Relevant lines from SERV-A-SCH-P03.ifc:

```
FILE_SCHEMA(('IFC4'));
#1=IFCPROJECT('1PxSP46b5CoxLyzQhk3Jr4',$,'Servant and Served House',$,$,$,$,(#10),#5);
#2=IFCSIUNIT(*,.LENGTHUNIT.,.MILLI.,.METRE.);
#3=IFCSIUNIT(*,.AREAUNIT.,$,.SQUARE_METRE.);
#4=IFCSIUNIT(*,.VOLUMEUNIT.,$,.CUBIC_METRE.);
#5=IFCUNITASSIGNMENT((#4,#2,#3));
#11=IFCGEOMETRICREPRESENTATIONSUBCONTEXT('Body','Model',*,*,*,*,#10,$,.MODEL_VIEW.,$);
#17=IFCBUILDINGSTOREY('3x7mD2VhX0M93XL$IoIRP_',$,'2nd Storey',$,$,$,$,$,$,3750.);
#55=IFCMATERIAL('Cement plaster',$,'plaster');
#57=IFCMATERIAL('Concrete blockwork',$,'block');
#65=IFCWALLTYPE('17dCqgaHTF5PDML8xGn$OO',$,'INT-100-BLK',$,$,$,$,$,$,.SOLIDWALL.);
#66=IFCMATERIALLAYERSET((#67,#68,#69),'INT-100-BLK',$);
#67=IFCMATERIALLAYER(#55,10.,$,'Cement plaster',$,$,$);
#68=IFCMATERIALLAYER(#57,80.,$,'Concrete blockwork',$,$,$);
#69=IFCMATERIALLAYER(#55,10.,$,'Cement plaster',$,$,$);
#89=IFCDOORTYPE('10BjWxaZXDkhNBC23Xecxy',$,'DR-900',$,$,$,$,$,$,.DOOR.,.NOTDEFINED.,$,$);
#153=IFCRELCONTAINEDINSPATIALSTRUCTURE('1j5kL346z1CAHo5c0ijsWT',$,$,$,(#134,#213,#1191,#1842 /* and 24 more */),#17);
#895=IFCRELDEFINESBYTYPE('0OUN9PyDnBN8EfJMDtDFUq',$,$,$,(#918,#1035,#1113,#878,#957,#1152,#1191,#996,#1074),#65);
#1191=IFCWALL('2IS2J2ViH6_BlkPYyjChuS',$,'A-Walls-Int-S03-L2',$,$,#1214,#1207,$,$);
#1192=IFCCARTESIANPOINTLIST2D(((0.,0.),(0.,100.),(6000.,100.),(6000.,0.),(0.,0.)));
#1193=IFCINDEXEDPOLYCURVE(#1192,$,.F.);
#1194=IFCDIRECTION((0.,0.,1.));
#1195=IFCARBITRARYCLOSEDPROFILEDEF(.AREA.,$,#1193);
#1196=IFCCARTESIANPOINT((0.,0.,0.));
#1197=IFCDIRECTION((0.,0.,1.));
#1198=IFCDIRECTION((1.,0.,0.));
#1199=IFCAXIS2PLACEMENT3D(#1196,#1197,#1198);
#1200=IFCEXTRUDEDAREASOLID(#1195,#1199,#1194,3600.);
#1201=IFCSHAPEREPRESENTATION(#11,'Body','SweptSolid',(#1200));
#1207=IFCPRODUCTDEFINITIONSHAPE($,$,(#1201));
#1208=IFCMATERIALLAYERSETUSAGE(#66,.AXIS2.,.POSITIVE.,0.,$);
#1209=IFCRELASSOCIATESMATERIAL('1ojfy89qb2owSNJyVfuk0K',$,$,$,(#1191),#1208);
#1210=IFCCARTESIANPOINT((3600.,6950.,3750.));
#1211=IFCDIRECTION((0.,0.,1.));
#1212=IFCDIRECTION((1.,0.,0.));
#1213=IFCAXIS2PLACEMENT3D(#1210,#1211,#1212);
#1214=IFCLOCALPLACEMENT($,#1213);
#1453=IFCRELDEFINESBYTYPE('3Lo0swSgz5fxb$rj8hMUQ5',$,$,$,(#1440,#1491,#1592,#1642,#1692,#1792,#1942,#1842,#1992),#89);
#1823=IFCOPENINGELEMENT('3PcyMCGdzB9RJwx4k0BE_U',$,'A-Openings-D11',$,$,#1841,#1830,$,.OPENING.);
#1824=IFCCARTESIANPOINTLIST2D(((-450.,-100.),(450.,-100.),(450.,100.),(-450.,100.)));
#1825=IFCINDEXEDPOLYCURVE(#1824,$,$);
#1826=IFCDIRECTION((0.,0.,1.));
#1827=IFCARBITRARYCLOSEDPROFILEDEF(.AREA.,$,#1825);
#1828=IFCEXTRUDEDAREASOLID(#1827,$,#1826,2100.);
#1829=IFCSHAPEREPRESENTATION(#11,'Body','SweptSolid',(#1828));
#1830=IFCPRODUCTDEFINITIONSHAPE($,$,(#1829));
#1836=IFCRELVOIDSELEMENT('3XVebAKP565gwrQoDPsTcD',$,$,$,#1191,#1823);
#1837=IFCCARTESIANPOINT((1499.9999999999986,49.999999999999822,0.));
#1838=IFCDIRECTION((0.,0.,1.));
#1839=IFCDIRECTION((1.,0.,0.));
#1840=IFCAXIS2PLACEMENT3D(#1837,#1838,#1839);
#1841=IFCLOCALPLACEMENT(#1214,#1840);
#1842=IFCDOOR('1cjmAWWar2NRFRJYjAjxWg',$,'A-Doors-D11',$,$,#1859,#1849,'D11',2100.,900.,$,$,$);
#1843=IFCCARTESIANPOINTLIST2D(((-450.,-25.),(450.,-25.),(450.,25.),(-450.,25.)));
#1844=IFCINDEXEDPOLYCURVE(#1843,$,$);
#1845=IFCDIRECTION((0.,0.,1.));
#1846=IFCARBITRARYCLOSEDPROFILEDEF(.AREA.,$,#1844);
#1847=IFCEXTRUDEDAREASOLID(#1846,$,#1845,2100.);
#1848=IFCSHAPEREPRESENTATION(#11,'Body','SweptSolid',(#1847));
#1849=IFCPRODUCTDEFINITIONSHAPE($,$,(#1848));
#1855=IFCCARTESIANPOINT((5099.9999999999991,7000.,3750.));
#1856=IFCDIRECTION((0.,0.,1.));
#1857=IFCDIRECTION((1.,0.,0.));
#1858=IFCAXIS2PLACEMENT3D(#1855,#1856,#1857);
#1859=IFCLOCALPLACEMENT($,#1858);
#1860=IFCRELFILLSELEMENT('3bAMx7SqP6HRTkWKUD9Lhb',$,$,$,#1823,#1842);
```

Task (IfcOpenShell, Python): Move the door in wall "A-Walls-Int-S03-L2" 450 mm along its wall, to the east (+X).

```python
import ifcopenshell
import ifcopenshell.api.geometry
import ifcopenshell.util.placement
import ifcopenshell.util.unit

model = ifcopenshell.open("SERV-A-SCH-P03.ifc")
unit_scale = ifcopenshell.util.unit.calculate_unit_scale(model)

door = model.by_guid("1cjmAWWar2NRFRJYjAjxWg")
opening = door.FillsVoids[0].RelatingOpeningElement
wall = opening.VoidsElements[0].RelatingBuildingElement

wall_matrix = ifcopenshell.util.placement.get_local_placement(wall.ObjectPlacement)
shift = wall_matrix[:3, 0] * 0.45 / unit_scale
before = ifcopenshell.util.placement.get_local_placement(door.ObjectPlacement)[:3, 3].copy()

# The door is not placed relative to its opening, so move both.
for product in (opening, door):
    matrix = ifcopenshell.util.placement.get_local_placement(product.ObjectPlacement)
    matrix[:3, 3] += shift
    ifcopenshell.api.geometry.edit_object_placement(model, product=product, matrix=matrix, is_si=False)

after = ifcopenshell.util.placement.get_local_placement(door.ObjectPlacement)[:3, 3]
print("door moved by", (after - before).round(3) + 0.0)

model.write("SERV-A-SCH-P03-out.ifc")
```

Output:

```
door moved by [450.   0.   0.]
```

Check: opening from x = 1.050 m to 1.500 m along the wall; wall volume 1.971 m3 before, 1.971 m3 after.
